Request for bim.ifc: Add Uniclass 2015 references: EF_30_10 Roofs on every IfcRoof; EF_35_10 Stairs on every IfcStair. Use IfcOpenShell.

First a look at what the model holds.

```python
import ifcopenshell

model = ifcopenshell.open("bim.ifc")
print(model.schema)
print("classifications:", [c.Name for c in model.by_type("IfcClassification")])
for ifc_class in ("IfcDoor", "IfcRoof", "IfcStair", "IfcWall", "IfcWindow"):
    print(ifc_class, len(model.by_type(ifc_class)))
```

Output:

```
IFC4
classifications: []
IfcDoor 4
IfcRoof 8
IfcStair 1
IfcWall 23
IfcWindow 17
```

```python
import ifcopenshell
import ifcopenshell.api.classification

model = ifcopenshell.open("bim.ifc")

system = ifcopenshell.api.classification.add_classification(model, classification="Uniclass 2015")

codes = {
    "IfcRoof": ("EF_30_10", "Roofs"),
    "IfcStair": ("EF_35_10", "Stairs"),
}
for ifc_class, (code, name) in codes.items():
    products = model.by_type(ifc_class)
    ifcopenshell.api.classification.add_reference(
        model, products=products, classification=system, identification=code, name=name
    )
    print(code, len(products))

model.write("bim_v2.ifc")
```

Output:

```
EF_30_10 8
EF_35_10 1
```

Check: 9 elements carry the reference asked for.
